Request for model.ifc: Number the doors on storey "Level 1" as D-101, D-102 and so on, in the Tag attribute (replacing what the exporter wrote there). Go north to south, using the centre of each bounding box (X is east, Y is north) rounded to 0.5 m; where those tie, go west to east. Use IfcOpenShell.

First a look at what the model holds.

```python
import ifcopenshell
import ifcopenshell.util.element
import ifcopenshell.util.placement

model = ifcopenshell.open("model.ifc")
print(model.schema)
storey = next(s for s in model.by_type("IfcBuildingStorey") if s.Name == "Level 1")
doors = [e for e in ifcopenshell.util.element.get_decomposition(storey) if e.is_a("IfcDoor")]
for e in sorted(doors, key=lambda e: e.id()):
    origin = ifcopenshell.util.placement.get_local_placement(e.ObjectPlacement)[:3, 3]
    print(e.id(), e.Tag, e.Name, origin.round(2) + 0.0, sep=" | ")
```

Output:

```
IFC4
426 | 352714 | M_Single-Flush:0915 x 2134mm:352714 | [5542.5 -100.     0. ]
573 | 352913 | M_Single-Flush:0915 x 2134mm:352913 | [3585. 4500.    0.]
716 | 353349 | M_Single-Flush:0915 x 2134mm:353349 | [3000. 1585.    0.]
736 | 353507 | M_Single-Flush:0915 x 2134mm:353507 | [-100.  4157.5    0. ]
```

```python
import ifcopenshell
import ifcopenshell.geom
import ifcopenshell.util.element
import ifcopenshell.util.shape

model = ifcopenshell.open("model.ifc")
settings = ifcopenshell.geom.settings()
settings.set("use-world-coords", True)


def centre(element):
    shape = ifcopenshell.geom.create_shape(settings, element)
    return ifcopenshell.util.shape.get_bbox_centroid(shape.geometry)


storey = next(s for s in model.by_type("IfcBuildingStorey") if s.Name == "Level 1")
doors = [e for e in ifcopenshell.util.element.get_decomposition(storey) if e.is_a("IfcDoor")]

# Insertion points can sit at a corner or the storey origin, so sort by the geometry (in metres).
centres = {e: centre(e) for e in doors}
doors.sort(key=lambda e: (-round(centres[e][1] / 0.5), centres[e][0]))

for i, e in enumerate(doors, start=1):
    number = f"D-1{i:02d}"
    e.Tag = number
    print(e.id(), number)

model.write("model_updated.ifc")
```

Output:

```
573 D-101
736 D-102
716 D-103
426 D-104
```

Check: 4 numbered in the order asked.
